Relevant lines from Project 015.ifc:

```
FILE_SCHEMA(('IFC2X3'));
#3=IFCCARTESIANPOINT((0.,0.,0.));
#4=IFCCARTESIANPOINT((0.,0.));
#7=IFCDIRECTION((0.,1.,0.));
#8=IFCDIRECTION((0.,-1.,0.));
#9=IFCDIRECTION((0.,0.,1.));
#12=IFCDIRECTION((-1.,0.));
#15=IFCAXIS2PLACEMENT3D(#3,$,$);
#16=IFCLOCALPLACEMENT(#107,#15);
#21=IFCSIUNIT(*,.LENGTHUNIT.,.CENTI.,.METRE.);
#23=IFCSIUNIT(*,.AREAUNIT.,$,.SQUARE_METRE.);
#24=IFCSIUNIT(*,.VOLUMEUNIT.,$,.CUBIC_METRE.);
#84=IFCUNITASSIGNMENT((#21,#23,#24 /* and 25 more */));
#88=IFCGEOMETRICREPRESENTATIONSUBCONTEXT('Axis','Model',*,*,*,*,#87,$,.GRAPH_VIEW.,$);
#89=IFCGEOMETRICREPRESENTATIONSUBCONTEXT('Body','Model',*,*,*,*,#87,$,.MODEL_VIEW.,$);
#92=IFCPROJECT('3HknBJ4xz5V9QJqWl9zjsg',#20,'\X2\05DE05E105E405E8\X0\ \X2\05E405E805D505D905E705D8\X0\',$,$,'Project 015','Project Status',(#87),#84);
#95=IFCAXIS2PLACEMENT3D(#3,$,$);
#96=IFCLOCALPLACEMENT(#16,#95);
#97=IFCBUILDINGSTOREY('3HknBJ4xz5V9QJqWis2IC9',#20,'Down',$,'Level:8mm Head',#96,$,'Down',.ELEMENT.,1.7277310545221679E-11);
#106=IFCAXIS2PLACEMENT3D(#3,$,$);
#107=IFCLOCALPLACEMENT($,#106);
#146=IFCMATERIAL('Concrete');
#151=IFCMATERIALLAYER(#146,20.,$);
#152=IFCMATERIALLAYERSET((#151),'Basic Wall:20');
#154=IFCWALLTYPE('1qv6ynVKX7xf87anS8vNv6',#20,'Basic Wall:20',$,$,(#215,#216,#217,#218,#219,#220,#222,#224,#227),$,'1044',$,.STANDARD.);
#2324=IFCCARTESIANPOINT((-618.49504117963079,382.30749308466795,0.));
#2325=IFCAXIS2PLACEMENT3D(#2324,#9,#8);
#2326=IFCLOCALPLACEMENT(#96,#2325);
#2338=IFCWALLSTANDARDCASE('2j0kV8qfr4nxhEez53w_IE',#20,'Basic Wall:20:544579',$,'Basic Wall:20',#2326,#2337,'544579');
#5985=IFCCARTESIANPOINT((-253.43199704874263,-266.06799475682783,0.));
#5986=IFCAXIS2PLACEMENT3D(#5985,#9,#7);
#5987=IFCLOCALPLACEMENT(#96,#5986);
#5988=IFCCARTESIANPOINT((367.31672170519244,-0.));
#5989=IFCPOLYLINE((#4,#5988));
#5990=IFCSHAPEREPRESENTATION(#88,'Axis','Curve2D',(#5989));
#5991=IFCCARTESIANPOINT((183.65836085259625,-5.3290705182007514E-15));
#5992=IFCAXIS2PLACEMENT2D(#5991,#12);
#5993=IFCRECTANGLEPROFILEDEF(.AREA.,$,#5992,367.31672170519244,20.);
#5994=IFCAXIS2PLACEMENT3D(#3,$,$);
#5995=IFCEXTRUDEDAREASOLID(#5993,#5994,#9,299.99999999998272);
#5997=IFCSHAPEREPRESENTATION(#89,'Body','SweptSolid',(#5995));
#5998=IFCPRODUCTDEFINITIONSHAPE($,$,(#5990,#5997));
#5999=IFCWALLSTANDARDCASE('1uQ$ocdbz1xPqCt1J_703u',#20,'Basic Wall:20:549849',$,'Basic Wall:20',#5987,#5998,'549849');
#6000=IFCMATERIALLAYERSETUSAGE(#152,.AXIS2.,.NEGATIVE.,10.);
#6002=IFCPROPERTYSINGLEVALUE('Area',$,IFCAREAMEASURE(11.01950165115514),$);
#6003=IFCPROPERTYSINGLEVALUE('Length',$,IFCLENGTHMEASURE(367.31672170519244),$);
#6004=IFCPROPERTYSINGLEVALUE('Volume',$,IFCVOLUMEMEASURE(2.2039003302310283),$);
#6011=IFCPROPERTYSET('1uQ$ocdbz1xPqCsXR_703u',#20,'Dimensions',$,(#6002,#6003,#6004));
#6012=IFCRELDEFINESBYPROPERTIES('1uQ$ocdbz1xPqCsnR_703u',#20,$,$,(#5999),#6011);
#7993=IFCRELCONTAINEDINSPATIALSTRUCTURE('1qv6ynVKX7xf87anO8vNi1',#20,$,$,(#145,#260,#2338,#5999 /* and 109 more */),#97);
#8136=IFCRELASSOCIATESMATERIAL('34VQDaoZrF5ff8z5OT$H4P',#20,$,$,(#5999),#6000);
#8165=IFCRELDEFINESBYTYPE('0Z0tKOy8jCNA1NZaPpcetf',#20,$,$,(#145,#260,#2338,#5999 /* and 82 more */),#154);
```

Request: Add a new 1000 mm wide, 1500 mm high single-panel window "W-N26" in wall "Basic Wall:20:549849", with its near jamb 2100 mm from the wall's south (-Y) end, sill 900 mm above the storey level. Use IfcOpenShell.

```python
import numpy as np
import ifcopenshell
import ifcopenshell.api.feature
import ifcopenshell.api.geometry
import ifcopenshell.api.pset
import ifcopenshell.api.root
import ifcopenshell.api.spatial
import ifcopenshell.api.type
import ifcopenshell.geom
import ifcopenshell.util.element
import ifcopenshell.util.placement
import ifcopenshell.util.representation
import ifcopenshell.util.shape
import ifcopenshell.util.unit

model = ifcopenshell.open("Project 015.ifc")
unit_scale = ifcopenshell.util.unit.calculate_unit_scale(model)
area_scale = ifcopenshell.util.unit.calculate_unit_scale(model, "AREAUNIT")
volume_scale = ifcopenshell.util.unit.calculate_unit_scale(model, "VOLUMEUNIT")
settings = ifcopenshell.geom.settings()


def volume(element):
    """Net volume in cubic metres, openings subtracted."""
    shape = ifcopenshell.geom.create_shape(settings, element)
    return ifcopenshell.util.shape.get_volume(shape.geometry)


wall = model.by_id(5999)
storey = ifcopenshell.util.element.get_container(wall, ifc_class="IfcBuildingStorey")
context = ifcopenshell.util.representation.get_context(model, "Model", "Body", "MODEL_VIEW")
before = volume(wall)

width, height, from_end, sill = 1, 1.5, 2.1, 0.9  # metres

# The wall runs along its own X axis, and the end named is its -X end.
wall_shape = ifcopenshell.geom.create_shape(settings, wall)
x, y, z = ifcopenshell.util.shape.get_vertices(wall_shape.geometry).T
start = x.min() + from_end
face, thickness = float(y.min()), float(y.max() - y.min())
wall_matrix = ifcopenshell.util.placement.get_local_placement(wall.ObjectPlacement)
level = ifcopenshell.util.placement.get_local_placement(storey.ObjectPlacement)[2, 3]


def in_wall(x, y):
    """Placement at x, y metres in the wall's axes, at sill height."""
    matrix = wall_matrix.copy()
    matrix[:, 3] = wall_matrix @ np.array([x / unit_scale, y / unit_scale, 0.0, 1.0])
    matrix[2, 3] = level + sill / unit_scale
    return matrix


# Opening: a box that overshoots both wall faces by 50 mm.
opening = ifcopenshell.api.root.create_entity(model, ifc_class="IfcOpeningElement")
box = ifcopenshell.api.geometry.add_wall_representation(
    model, context=context, length=width, height=height, thickness=thickness + 0.1
)
ifcopenshell.api.geometry.assign_representation(model, product=opening, representation=box)
ifcopenshell.api.geometry.edit_object_placement(model, product=opening, matrix=in_wall(start, face - 0.05), is_si=False)
ifcopenshell.api.feature.add_feature(model, feature=opening, element=wall)

window = ifcopenshell.api.root.create_entity(model, ifc_class="IfcWindow", name="W-N26")
window.OverallWidth, window.OverallHeight = width / unit_scale, height / unit_scale
body = ifcopenshell.api.geometry.add_window_representation(
    model,
    context=context,
    overall_width=window.OverallWidth,
    overall_height=window.OverallHeight,
    partition_type="SINGLE_PANEL",
)
ifcopenshell.api.geometry.assign_representation(model, product=window, representation=body)
ifcopenshell.api.spatial.assign_container(model, products=[window], relating_structure=storey)
fills = ifcopenshell.api.feature.add_filling(model, opening=opening, element=window)
fills.OwnerHistory = window.OwnerHistory  # required in IFC2X3

# IFC2X3 keeps the operation on the window style.
style = ifcopenshell.api.root.create_entity(model, ifc_class="IfcWindowStyle", name="W-N26")
style.OperationType, style.ConstructionType = "SINGLE_PANEL", "NOTDEFINED"
style.ParameterTakesPrecedence = style.Sizeable = False
ifcopenshell.api.type.assign_type(model, related_objects=[window], relating_type=style)

# Centre the window in the wall's thickness.
ifcopenshell.api.geometry.edit_object_placement(model, product=window, matrix=in_wall(start, face), is_si=False)
window_shape = ifcopenshell.geom.create_shape(settings, window)
depth = ifcopenshell.util.shape.get_vertices(window_shape.geometry)[:, 1]
offset = face + thickness / 2 - (depth.min() + depth.max()) / 2
ifcopenshell.api.geometry.edit_object_placement(model, product=window, matrix=in_wall(start, offset), is_si=False)

after = volume(wall)

# Update the wall's stored quantities.
pset = model.by_id(ifcopenshell.util.element.get_pset(wall, "Dimensions", should_inherit=False)["id"])
ifcopenshell.api.pset.edit_pset(model, pset=pset, properties={
    "Area": model.create_entity("IfcAreaMeasure", after / thickness / area_scale),
    "Volume": model.create_entity("IfcVolumeMeasure", after / volume_scale),
})

print(f"wall volume {before:.3f} -> {after:.3f} m3")

model.write("Project 015_edited.ifc")
```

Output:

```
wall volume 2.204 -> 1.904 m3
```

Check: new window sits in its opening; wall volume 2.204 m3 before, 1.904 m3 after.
